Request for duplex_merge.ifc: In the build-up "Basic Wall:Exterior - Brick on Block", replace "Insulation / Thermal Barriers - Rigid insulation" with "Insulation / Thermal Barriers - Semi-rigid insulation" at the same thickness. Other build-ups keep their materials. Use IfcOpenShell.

First a look at what the model holds.

```python
import ifcopenshell
import ifcopenshell.util.element

model = ifcopenshell.open("duplex_merge.ifc")
print(model.schema)
for layer_set in model.by_type("IfcMaterialLayerSet"):
    if layer_set.LayerSetName == "Basic Wall:Exterior - Brick on Block":
        for layer in layer_set.MaterialLayers:
            print(layer.id(), layer.Material and layer.Material.Name, layer.LayerThickness, sep=" | ")
        print(len(ifcopenshell.util.element.get_elements_by_material(model, layer_set)), "elements and types use it")
print(sorted(m.Name for m in model.by_type("IfcMaterial") if m.Name)[:60])
```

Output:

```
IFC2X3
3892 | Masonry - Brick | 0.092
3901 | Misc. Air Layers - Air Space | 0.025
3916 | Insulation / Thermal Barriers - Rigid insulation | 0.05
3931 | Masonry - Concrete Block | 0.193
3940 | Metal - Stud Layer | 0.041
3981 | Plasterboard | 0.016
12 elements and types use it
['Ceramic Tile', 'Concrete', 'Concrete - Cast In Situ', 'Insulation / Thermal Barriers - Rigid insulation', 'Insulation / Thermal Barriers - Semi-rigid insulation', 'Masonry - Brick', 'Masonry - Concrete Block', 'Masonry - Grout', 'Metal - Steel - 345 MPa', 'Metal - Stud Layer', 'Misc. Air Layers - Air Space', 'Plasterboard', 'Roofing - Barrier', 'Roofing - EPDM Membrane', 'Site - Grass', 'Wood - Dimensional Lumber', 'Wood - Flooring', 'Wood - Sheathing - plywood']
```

```python
import ifcopenshell
import ifcopenshell.api.material

model = ifcopenshell.open("duplex_merge.ifc")

layer_set = next(s for s in model.by_type("IfcMaterialLayerSet") if s.LayerSetName == "Basic Wall:Exterior - Brick on Block")
layer = next(l for l in layer_set.MaterialLayers if l.Material and l.Material.Name == "Insulation / Thermal Barriers - Rigid insulation")
material = next(m for m in model.by_type("IfcMaterial") if m.Name == "Insulation / Thermal Barriers - Semi-rigid insulation")

# Point this one layer at the other material; renaming the old one would change it everywhere.
ifcopenshell.api.material.edit_layer(model, layer=layer, attributes={}, material=material)

print([l.Material.Name if l.Material else None for l in layer_set.MaterialLayers])

model.write("duplex_merge_edited.ifc")
```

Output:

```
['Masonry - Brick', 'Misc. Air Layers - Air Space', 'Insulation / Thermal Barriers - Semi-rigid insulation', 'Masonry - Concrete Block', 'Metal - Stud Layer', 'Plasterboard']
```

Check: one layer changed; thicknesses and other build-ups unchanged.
